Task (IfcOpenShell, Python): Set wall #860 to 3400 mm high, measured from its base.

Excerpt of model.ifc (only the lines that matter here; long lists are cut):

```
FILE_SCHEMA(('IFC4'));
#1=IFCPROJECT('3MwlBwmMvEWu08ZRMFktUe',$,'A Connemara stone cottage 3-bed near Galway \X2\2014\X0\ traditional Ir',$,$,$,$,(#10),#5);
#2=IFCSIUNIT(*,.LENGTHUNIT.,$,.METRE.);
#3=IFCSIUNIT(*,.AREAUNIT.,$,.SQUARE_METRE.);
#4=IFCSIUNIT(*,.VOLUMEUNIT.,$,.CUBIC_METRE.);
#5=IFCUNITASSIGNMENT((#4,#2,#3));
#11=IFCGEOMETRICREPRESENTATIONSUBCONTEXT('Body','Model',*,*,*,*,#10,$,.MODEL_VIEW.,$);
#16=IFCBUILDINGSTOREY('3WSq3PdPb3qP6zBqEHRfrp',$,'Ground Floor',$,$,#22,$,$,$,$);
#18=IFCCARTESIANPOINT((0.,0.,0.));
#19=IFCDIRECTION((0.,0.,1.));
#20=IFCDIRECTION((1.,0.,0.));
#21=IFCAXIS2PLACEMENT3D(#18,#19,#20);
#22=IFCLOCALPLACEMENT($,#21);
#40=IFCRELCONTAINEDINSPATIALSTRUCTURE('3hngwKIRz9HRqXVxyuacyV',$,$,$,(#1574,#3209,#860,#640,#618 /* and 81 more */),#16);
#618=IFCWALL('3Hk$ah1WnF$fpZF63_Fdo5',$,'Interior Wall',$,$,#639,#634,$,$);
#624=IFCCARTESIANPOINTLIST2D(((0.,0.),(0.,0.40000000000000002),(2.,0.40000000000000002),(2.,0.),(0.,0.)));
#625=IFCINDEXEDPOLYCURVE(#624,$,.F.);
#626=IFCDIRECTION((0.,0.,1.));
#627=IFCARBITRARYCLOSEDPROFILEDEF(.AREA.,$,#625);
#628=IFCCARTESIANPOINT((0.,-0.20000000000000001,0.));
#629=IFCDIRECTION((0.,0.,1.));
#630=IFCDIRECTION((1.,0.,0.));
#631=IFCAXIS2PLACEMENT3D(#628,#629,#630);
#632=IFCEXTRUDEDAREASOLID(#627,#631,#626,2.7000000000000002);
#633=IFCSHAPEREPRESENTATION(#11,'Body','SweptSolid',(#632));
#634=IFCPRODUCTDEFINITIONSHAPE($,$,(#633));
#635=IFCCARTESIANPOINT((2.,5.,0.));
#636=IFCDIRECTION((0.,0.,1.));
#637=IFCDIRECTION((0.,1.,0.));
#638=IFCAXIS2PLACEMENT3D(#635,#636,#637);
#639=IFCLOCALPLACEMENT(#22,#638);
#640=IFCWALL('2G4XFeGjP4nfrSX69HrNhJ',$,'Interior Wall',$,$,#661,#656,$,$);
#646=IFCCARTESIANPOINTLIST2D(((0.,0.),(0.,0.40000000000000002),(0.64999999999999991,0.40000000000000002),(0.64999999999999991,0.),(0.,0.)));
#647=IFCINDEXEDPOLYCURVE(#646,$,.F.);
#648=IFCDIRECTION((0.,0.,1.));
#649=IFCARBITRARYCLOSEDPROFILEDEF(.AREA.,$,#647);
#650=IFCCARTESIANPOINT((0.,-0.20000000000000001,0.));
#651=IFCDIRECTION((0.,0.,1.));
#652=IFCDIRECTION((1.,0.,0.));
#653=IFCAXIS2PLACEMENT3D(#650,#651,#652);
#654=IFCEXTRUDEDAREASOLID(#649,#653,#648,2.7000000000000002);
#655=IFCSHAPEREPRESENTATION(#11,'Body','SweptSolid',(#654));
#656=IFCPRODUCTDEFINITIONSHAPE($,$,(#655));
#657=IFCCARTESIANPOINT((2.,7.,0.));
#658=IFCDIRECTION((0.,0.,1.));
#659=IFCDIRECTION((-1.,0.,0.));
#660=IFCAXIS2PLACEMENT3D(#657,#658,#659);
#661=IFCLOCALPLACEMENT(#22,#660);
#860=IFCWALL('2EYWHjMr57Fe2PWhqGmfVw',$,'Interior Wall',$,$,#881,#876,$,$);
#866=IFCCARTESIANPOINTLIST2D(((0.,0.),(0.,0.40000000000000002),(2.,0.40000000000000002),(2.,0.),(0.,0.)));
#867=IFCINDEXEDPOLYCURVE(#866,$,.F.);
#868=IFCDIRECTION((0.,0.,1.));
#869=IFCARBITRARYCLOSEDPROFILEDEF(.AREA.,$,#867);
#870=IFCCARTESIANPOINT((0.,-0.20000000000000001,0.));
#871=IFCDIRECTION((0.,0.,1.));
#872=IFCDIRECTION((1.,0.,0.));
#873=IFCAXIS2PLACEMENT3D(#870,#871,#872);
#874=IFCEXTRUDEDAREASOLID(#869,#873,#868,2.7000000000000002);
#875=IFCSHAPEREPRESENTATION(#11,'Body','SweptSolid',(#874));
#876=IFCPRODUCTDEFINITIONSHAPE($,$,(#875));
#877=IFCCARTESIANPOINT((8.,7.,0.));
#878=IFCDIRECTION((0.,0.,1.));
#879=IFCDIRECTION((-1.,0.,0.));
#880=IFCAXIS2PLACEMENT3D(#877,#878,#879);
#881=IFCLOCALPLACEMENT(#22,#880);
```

```python
import ifcopenshell
import ifcopenshell.geom
import ifcopenshell.util.representation
import ifcopenshell.util.shape
import ifcopenshell.util.unit

model = ifcopenshell.open("model.ifc")
unit_scale = ifcopenshell.util.unit.calculate_unit_scale(model)
settings = ifcopenshell.geom.settings()


def volume(element):
    """Net volume in cubic metres, openings subtracted."""
    shape = ifcopenshell.geom.create_shape(settings, element)
    return ifcopenshell.util.shape.get_volume(shape.geometry)


wall = model.by_guid("2EYWHjMr57Fe2PWhqGmfVw")
before = volume(wall)

body = ifcopenshell.util.representation.get_representation(wall, "Model", "Body")
solid = body.Items[0]
old_height = solid.Depth
solid.Depth = 3.4 / unit_scale
after = volume(wall)

print(f"height {old_height:g} -> {solid.Depth:g}, volume {before:.3f} -> {after:.3f} m3")

model.write("model_rev.ifc")
```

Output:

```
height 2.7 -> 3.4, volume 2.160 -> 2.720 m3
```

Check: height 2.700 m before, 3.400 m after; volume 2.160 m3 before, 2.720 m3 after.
